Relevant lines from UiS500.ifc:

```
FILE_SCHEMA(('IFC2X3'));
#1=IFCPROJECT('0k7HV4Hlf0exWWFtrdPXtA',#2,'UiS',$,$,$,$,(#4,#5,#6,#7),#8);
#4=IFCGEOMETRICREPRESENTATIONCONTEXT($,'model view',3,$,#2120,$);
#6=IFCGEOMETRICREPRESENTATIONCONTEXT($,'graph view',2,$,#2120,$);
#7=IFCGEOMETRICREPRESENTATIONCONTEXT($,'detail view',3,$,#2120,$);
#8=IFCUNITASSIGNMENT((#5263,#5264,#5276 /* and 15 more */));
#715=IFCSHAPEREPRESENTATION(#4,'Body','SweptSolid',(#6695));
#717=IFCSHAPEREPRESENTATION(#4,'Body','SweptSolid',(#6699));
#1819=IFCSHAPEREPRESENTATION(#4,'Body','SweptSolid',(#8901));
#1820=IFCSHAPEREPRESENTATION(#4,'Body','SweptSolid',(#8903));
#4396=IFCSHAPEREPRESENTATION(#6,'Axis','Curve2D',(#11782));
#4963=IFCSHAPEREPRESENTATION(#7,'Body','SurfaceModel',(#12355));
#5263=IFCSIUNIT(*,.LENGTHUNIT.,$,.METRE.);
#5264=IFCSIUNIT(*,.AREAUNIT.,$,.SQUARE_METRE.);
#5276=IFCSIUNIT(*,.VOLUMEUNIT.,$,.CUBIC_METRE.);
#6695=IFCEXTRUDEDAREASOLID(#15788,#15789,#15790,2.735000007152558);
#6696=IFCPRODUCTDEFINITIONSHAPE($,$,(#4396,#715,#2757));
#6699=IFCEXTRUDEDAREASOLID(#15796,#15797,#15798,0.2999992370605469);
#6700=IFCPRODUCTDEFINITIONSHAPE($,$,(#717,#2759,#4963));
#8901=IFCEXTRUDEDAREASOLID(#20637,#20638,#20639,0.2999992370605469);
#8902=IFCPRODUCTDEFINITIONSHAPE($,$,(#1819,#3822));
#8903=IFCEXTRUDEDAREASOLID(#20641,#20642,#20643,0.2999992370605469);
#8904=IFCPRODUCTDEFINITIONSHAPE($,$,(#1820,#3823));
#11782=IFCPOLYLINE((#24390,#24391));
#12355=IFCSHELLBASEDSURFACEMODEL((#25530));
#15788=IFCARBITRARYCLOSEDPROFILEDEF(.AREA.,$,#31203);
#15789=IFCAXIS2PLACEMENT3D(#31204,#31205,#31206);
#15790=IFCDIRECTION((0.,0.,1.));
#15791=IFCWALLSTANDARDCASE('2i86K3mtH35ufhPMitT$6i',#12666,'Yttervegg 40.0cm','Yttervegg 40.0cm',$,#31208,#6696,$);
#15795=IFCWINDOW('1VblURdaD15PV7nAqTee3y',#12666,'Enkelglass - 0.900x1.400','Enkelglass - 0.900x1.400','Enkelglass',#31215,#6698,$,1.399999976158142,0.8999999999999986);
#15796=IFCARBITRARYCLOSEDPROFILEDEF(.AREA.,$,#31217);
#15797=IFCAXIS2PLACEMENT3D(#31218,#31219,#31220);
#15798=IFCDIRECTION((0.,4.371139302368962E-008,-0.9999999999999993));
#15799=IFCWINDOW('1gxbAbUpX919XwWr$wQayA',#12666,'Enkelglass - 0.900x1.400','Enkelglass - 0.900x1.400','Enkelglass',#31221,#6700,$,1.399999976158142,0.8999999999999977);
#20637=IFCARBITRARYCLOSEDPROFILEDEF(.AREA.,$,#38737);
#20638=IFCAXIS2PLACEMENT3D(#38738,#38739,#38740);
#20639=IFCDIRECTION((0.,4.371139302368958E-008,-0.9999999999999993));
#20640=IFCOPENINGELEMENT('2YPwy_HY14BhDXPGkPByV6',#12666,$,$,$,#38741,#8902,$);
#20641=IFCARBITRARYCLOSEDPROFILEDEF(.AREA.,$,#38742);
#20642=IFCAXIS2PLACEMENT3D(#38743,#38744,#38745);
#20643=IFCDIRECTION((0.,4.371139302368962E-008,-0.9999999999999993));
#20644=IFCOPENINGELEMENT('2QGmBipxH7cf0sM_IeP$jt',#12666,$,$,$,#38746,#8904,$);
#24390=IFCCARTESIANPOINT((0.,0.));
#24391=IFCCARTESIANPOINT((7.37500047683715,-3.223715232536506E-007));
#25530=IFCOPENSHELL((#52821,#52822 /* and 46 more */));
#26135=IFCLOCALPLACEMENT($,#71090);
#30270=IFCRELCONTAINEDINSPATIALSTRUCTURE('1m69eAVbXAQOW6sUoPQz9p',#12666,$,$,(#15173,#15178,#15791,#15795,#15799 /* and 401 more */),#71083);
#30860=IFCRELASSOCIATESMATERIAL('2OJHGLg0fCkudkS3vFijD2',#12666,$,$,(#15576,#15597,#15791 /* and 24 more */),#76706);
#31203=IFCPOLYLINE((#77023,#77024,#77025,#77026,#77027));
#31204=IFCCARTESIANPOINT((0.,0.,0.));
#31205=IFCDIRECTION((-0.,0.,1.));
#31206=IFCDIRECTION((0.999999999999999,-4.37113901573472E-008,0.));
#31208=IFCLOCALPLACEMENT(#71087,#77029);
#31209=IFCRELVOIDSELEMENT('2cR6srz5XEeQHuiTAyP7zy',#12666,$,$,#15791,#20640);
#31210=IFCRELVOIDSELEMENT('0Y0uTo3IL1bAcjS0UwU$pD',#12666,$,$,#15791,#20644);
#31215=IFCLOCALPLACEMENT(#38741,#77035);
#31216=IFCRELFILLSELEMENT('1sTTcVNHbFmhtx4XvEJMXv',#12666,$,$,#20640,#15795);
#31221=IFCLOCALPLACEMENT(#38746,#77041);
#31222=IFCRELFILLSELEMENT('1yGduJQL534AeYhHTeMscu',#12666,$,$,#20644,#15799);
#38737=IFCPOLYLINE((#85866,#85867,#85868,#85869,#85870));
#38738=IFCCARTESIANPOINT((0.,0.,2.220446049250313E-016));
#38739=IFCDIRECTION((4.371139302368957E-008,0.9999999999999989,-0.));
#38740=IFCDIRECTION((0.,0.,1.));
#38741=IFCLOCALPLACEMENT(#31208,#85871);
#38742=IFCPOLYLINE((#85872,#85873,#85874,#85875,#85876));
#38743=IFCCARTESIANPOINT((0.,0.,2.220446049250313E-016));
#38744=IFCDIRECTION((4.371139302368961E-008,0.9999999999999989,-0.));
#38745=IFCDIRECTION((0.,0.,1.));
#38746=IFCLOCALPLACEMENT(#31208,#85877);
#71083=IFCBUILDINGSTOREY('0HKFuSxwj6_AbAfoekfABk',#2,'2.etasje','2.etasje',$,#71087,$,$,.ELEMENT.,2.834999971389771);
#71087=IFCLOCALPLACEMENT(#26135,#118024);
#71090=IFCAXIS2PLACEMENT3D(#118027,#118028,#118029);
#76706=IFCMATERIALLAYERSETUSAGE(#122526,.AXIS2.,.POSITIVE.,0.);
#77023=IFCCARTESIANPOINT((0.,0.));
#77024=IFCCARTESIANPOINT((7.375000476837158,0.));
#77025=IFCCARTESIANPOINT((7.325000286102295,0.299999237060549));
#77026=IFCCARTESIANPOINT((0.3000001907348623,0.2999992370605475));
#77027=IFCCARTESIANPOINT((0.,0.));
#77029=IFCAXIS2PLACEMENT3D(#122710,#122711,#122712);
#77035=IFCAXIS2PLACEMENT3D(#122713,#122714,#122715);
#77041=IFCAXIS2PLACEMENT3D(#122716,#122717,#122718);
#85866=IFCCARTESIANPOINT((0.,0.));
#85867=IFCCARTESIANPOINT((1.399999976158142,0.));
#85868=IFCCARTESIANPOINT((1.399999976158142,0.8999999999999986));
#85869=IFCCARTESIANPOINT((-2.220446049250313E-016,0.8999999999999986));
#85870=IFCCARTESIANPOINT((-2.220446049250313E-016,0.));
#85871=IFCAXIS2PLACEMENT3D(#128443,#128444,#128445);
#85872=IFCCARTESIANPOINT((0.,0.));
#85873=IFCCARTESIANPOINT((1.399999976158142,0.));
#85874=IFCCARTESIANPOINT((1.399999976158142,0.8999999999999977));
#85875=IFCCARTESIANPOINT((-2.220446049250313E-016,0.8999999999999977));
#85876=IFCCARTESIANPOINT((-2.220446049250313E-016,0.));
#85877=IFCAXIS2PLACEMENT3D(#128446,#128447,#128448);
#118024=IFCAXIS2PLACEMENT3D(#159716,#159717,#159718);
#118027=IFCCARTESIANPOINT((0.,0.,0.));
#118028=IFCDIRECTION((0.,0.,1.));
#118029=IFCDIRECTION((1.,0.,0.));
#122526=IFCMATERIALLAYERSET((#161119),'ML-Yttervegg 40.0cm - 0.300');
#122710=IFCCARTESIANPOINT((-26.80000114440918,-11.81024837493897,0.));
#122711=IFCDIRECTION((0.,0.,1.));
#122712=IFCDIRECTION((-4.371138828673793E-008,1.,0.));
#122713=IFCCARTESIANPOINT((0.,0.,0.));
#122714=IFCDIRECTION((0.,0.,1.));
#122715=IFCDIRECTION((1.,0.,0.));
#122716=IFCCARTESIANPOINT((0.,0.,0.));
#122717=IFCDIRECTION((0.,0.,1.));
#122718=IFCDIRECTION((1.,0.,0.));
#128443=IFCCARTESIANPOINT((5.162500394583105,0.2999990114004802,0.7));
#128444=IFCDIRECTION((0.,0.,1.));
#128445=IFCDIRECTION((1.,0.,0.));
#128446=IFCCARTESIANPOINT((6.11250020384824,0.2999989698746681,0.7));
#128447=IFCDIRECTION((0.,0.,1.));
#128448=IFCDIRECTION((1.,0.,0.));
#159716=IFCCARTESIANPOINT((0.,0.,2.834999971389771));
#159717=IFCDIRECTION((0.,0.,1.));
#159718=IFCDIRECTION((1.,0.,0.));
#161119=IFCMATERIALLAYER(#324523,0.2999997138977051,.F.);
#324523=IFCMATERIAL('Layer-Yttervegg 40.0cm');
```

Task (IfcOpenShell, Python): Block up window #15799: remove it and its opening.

```python
import ifcopenshell
import ifcopenshell.api.feature
import ifcopenshell.api.root
import ifcopenshell.geom
import ifcopenshell.util.shape

model = ifcopenshell.open("UiS500.ifc")
settings = ifcopenshell.geom.settings()


def volume(element):
    """Net volume in cubic metres, openings subtracted."""
    shape = ifcopenshell.geom.create_shape(settings, element)
    return ifcopenshell.util.shape.get_volume(shape.geometry)


window = model.by_id(15799)
opening = window.FillsVoids[0].RelatingOpeningElement
wall = opening.VoidsElements[0].RelatingBuildingElement
before = volume(wall)

ifcopenshell.api.root.remove_product(model, product=window)
ifcopenshell.api.feature.remove_feature(model, feature=opening)

after = volume(wall)

print(f"wall volume {before:.3f} -> {after:.3f} m3")

model.write("UiS500_updated.ifc")
```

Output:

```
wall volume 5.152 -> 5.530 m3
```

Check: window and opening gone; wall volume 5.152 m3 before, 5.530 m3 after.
